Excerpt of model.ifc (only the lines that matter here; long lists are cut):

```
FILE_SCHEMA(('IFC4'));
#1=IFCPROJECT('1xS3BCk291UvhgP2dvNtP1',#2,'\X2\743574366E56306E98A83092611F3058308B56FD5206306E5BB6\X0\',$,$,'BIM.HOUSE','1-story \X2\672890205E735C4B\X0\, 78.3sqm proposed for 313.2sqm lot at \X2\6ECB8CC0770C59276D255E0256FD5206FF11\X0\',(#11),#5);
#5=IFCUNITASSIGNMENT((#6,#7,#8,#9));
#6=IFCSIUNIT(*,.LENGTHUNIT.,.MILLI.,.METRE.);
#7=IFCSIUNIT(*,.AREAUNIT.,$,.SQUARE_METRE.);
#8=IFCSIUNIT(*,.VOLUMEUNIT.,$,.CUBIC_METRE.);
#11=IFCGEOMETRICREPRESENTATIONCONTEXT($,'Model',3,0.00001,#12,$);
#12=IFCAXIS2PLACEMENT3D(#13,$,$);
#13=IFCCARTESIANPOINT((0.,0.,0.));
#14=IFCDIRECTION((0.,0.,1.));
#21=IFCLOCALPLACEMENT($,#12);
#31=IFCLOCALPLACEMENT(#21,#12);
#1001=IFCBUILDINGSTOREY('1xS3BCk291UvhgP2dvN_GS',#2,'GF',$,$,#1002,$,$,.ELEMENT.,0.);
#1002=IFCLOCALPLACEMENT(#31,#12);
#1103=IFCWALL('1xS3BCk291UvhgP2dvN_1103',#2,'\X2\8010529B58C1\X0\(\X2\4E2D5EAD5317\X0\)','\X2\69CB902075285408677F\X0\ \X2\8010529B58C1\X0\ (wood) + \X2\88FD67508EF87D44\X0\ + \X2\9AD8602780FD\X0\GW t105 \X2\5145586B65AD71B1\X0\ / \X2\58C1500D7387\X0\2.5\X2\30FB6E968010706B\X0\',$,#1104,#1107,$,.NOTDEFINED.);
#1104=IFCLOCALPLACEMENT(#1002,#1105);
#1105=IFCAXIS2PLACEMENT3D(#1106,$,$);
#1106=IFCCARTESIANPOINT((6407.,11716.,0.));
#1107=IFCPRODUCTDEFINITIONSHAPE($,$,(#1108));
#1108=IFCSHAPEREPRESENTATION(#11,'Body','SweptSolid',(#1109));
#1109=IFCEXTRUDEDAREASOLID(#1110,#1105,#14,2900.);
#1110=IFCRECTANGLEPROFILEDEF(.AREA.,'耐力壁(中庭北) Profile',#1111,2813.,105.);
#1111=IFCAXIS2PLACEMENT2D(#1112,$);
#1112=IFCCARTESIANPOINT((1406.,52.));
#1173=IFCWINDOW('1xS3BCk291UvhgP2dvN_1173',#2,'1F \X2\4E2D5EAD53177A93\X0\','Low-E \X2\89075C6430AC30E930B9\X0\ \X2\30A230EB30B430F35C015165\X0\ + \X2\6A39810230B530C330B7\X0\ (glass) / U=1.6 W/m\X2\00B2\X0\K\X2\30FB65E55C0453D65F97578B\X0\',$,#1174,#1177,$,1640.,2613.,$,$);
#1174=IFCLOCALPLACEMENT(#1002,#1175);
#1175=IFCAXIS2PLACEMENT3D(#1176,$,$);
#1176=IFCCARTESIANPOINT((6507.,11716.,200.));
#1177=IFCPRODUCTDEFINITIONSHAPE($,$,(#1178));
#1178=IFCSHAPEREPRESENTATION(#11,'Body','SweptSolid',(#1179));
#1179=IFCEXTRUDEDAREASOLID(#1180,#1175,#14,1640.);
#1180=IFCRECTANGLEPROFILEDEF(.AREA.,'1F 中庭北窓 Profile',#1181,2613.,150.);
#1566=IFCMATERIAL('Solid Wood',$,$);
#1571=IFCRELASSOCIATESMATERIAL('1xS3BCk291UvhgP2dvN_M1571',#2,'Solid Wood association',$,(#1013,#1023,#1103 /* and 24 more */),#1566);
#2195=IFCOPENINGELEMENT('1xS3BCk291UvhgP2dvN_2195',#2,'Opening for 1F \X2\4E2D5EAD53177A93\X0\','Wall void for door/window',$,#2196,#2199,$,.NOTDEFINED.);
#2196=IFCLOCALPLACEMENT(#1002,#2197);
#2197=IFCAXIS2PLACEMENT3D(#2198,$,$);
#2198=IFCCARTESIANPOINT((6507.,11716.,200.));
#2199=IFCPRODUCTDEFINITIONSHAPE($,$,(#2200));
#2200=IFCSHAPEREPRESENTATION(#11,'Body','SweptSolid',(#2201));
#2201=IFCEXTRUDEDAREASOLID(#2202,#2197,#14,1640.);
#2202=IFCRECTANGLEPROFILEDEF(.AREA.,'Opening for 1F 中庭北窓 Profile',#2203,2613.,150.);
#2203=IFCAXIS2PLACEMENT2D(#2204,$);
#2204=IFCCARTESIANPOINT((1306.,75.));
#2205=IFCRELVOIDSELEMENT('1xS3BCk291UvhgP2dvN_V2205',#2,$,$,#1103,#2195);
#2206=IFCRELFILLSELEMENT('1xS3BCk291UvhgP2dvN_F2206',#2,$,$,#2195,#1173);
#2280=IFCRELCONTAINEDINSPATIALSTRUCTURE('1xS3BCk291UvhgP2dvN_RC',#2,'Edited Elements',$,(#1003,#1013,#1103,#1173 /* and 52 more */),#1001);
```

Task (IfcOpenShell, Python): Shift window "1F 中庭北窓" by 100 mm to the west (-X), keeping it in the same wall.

```python
import ifcopenshell
import ifcopenshell.api.geometry
import ifcopenshell.util.placement

model = ifcopenshell.open("model.ifc")

window = model.by_id(1173)
opening = window.FillsVoids[0].RelatingOpeningElement
wall = opening.VoidsElements[0].RelatingBuildingElement

wall_matrix = ifcopenshell.util.placement.get_local_placement(wall.ObjectPlacement)
shift = wall_matrix[:3, 0] * -100.0
before = ifcopenshell.util.placement.get_local_placement(window.ObjectPlacement)[:3, 3].copy()

# The window is not placed relative to its opening, so move both.
for product in (opening, window):
    matrix = ifcopenshell.util.placement.get_local_placement(product.ObjectPlacement)
    matrix[:3, 3] += shift
    ifcopenshell.api.geometry.edit_object_placement(model, product=product, matrix=matrix, is_si=False)

after = ifcopenshell.util.placement.get_local_placement(window.ObjectPlacement)[:3, 3]
print("window moved by", (after - before).round(3) + 0.0)

model.write("model_edited.ifc")
```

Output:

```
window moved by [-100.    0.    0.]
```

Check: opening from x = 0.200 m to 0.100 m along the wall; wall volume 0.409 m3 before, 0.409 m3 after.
